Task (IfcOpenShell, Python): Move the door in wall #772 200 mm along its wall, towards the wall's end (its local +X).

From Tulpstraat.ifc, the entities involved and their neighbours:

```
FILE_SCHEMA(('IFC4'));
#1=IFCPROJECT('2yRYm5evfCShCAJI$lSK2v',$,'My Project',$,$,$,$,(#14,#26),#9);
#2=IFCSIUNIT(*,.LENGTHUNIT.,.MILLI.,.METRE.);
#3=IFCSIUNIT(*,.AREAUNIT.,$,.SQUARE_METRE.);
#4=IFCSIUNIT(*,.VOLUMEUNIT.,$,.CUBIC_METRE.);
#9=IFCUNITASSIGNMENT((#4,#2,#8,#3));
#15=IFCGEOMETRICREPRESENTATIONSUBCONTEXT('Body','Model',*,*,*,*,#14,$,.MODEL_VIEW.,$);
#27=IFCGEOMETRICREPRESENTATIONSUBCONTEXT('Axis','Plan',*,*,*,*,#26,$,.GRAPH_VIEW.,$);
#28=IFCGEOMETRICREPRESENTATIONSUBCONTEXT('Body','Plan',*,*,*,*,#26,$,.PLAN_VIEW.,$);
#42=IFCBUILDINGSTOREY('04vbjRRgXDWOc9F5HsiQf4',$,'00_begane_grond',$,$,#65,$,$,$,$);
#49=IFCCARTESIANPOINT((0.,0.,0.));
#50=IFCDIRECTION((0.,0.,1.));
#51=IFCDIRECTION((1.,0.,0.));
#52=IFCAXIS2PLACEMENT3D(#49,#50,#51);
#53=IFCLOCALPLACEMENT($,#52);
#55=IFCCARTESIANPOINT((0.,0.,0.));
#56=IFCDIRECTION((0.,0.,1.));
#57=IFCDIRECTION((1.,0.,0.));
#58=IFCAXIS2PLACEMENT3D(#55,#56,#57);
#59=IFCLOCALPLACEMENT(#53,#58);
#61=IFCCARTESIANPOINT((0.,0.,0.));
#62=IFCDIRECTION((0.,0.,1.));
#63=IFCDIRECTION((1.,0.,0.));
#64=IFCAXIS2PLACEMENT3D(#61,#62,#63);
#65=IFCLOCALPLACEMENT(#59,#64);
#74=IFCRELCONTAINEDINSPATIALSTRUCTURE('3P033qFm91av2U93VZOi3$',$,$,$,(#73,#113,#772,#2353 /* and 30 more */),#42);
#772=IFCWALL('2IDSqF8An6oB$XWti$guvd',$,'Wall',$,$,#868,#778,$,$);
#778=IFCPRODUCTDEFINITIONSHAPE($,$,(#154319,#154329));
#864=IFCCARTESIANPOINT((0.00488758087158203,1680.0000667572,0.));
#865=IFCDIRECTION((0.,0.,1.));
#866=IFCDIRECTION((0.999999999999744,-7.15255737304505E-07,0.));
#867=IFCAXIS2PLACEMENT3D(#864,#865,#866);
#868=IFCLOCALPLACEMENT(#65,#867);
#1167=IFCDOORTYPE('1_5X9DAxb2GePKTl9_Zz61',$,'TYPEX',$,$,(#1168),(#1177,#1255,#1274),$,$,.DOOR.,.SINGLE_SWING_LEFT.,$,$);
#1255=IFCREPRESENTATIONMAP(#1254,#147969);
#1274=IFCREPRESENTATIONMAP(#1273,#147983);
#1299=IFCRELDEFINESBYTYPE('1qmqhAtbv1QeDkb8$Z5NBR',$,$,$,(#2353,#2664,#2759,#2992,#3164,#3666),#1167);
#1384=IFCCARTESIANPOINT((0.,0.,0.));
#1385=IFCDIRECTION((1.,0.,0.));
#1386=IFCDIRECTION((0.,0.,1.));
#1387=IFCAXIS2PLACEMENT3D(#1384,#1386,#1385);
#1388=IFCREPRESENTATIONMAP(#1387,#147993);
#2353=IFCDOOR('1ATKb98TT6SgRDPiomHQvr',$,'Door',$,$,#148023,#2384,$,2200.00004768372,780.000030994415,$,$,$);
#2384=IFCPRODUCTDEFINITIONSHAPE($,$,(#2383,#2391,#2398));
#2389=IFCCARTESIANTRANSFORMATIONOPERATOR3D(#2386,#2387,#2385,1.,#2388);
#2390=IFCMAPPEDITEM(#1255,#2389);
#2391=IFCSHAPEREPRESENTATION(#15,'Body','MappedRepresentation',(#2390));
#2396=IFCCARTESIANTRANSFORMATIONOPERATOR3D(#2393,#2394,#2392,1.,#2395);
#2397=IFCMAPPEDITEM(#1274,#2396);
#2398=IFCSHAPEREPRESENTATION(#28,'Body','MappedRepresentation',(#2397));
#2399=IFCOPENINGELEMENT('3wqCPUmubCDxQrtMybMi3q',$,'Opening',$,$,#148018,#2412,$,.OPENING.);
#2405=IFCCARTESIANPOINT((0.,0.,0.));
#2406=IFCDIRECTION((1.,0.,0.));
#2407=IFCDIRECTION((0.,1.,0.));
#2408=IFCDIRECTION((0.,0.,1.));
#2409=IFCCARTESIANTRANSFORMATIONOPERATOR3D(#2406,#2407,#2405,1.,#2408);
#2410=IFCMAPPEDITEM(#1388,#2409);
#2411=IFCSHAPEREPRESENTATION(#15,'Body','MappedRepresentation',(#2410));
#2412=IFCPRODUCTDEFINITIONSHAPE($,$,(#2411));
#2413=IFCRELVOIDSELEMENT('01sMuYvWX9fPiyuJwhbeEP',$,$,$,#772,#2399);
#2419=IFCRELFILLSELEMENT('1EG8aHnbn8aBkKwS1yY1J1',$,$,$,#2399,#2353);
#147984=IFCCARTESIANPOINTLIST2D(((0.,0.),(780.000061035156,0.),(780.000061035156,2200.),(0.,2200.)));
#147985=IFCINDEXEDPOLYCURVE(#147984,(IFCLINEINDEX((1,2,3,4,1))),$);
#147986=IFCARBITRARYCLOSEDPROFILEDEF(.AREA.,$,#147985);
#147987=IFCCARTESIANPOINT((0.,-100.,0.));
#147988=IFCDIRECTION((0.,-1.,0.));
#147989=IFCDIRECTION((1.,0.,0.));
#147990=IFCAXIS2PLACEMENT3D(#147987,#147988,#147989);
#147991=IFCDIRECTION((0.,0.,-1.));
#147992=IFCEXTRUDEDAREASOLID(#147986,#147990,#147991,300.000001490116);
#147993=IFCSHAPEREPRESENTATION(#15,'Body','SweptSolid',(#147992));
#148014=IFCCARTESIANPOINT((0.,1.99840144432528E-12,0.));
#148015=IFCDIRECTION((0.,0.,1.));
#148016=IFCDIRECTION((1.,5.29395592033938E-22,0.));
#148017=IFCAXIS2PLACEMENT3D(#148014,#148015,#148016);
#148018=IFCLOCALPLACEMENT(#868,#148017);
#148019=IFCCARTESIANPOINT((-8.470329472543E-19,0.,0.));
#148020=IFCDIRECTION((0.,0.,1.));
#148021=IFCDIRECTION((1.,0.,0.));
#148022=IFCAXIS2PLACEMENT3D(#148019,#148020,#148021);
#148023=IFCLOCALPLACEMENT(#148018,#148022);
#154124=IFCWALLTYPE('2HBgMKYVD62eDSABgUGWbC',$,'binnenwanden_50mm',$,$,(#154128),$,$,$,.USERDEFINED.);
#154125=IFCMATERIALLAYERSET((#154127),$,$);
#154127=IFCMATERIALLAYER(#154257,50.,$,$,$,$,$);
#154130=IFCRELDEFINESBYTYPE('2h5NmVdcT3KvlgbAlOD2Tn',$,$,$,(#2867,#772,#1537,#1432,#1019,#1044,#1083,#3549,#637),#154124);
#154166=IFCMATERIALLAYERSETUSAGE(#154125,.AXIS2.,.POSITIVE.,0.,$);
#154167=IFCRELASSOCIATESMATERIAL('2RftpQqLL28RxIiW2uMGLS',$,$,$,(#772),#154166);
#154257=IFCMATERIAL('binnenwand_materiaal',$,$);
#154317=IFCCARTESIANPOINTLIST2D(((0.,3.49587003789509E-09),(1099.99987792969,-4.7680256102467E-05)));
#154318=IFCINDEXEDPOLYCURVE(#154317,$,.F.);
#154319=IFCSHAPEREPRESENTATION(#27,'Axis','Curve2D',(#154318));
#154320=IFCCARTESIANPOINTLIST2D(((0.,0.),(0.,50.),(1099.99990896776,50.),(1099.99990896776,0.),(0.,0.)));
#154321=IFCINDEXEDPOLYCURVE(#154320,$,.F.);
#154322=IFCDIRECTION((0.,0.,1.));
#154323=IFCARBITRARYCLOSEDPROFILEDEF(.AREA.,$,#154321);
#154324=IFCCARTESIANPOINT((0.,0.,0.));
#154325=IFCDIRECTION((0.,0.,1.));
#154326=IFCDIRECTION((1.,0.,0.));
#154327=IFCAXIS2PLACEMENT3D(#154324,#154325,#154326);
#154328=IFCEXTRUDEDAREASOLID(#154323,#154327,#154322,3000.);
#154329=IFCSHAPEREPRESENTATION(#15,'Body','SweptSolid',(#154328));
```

```python
import ifcopenshell
import ifcopenshell.api.geometry
import ifcopenshell.util.placement
import ifcopenshell.util.unit

model = ifcopenshell.open("Tulpstraat.ifc")
unit_scale = ifcopenshell.util.unit.calculate_unit_scale(model)

door = model.by_guid("1ATKb98TT6SgRDPiomHQvr")
opening = door.FillsVoids[0].RelatingOpeningElement
wall = opening.VoidsElements[0].RelatingBuildingElement

wall_matrix = ifcopenshell.util.placement.get_local_placement(wall.ObjectPlacement)
shift = wall_matrix[:3, 0] * 0.2 / unit_scale
before = ifcopenshell.util.placement.get_local_placement(door.ObjectPlacement)[:3, 3].copy()

# The door is placed relative to its opening, so it follows when the opening moves.
matrix = ifcopenshell.util.placement.get_local_placement(opening.ObjectPlacement)
matrix[:3, 3] += shift
ifcopenshell.api.geometry.edit_object_placement(
    model, product=opening, matrix=matrix, is_si=False, should_transform_children=True
)

after = ifcopenshell.util.placement.get_local_placement(door.ObjectPlacement)[:3, 3]
print("door moved by", (after - before).round(3) + 0.0)

model.write("Tulpstraat_edited.ifc")
```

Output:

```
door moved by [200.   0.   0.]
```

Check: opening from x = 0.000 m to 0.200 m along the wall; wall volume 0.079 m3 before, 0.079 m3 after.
